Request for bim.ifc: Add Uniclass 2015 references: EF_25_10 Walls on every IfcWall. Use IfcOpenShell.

First a look at what the model holds.

```python
import ifcopenshell

model = ifcopenshell.open("bim.ifc")
print(model.schema)
print("classifications:", [c.Name for c in model.by_type("IfcClassification")])
for ifc_class in ("IfcDoor", "IfcRoof", "IfcStair", "IfcWall", "IfcWindow"):
    print(ifc_class, len(model.by_type(ifc_class)))
```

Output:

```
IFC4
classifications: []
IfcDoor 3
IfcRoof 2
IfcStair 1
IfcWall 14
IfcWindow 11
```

```python
import ifcopenshell
import ifcopenshell.api.classification

model = ifcopenshell.open("bim.ifc")

system = ifcopenshell.api.classification.add_classification(model, classification="Uniclass 2015")

codes = {
    "IfcWall": ("EF_25_10", "Walls"),
}
for ifc_class, (code, name) in codes.items():
    products = model.by_type(ifc_class)
    ifcopenshell.api.classification.add_reference(
        model, products=products, classification=system, identification=code, name=name
    )
    print(code, len(products))

model.write("bim_updated.ifc")
```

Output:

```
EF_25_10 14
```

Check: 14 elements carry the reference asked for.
